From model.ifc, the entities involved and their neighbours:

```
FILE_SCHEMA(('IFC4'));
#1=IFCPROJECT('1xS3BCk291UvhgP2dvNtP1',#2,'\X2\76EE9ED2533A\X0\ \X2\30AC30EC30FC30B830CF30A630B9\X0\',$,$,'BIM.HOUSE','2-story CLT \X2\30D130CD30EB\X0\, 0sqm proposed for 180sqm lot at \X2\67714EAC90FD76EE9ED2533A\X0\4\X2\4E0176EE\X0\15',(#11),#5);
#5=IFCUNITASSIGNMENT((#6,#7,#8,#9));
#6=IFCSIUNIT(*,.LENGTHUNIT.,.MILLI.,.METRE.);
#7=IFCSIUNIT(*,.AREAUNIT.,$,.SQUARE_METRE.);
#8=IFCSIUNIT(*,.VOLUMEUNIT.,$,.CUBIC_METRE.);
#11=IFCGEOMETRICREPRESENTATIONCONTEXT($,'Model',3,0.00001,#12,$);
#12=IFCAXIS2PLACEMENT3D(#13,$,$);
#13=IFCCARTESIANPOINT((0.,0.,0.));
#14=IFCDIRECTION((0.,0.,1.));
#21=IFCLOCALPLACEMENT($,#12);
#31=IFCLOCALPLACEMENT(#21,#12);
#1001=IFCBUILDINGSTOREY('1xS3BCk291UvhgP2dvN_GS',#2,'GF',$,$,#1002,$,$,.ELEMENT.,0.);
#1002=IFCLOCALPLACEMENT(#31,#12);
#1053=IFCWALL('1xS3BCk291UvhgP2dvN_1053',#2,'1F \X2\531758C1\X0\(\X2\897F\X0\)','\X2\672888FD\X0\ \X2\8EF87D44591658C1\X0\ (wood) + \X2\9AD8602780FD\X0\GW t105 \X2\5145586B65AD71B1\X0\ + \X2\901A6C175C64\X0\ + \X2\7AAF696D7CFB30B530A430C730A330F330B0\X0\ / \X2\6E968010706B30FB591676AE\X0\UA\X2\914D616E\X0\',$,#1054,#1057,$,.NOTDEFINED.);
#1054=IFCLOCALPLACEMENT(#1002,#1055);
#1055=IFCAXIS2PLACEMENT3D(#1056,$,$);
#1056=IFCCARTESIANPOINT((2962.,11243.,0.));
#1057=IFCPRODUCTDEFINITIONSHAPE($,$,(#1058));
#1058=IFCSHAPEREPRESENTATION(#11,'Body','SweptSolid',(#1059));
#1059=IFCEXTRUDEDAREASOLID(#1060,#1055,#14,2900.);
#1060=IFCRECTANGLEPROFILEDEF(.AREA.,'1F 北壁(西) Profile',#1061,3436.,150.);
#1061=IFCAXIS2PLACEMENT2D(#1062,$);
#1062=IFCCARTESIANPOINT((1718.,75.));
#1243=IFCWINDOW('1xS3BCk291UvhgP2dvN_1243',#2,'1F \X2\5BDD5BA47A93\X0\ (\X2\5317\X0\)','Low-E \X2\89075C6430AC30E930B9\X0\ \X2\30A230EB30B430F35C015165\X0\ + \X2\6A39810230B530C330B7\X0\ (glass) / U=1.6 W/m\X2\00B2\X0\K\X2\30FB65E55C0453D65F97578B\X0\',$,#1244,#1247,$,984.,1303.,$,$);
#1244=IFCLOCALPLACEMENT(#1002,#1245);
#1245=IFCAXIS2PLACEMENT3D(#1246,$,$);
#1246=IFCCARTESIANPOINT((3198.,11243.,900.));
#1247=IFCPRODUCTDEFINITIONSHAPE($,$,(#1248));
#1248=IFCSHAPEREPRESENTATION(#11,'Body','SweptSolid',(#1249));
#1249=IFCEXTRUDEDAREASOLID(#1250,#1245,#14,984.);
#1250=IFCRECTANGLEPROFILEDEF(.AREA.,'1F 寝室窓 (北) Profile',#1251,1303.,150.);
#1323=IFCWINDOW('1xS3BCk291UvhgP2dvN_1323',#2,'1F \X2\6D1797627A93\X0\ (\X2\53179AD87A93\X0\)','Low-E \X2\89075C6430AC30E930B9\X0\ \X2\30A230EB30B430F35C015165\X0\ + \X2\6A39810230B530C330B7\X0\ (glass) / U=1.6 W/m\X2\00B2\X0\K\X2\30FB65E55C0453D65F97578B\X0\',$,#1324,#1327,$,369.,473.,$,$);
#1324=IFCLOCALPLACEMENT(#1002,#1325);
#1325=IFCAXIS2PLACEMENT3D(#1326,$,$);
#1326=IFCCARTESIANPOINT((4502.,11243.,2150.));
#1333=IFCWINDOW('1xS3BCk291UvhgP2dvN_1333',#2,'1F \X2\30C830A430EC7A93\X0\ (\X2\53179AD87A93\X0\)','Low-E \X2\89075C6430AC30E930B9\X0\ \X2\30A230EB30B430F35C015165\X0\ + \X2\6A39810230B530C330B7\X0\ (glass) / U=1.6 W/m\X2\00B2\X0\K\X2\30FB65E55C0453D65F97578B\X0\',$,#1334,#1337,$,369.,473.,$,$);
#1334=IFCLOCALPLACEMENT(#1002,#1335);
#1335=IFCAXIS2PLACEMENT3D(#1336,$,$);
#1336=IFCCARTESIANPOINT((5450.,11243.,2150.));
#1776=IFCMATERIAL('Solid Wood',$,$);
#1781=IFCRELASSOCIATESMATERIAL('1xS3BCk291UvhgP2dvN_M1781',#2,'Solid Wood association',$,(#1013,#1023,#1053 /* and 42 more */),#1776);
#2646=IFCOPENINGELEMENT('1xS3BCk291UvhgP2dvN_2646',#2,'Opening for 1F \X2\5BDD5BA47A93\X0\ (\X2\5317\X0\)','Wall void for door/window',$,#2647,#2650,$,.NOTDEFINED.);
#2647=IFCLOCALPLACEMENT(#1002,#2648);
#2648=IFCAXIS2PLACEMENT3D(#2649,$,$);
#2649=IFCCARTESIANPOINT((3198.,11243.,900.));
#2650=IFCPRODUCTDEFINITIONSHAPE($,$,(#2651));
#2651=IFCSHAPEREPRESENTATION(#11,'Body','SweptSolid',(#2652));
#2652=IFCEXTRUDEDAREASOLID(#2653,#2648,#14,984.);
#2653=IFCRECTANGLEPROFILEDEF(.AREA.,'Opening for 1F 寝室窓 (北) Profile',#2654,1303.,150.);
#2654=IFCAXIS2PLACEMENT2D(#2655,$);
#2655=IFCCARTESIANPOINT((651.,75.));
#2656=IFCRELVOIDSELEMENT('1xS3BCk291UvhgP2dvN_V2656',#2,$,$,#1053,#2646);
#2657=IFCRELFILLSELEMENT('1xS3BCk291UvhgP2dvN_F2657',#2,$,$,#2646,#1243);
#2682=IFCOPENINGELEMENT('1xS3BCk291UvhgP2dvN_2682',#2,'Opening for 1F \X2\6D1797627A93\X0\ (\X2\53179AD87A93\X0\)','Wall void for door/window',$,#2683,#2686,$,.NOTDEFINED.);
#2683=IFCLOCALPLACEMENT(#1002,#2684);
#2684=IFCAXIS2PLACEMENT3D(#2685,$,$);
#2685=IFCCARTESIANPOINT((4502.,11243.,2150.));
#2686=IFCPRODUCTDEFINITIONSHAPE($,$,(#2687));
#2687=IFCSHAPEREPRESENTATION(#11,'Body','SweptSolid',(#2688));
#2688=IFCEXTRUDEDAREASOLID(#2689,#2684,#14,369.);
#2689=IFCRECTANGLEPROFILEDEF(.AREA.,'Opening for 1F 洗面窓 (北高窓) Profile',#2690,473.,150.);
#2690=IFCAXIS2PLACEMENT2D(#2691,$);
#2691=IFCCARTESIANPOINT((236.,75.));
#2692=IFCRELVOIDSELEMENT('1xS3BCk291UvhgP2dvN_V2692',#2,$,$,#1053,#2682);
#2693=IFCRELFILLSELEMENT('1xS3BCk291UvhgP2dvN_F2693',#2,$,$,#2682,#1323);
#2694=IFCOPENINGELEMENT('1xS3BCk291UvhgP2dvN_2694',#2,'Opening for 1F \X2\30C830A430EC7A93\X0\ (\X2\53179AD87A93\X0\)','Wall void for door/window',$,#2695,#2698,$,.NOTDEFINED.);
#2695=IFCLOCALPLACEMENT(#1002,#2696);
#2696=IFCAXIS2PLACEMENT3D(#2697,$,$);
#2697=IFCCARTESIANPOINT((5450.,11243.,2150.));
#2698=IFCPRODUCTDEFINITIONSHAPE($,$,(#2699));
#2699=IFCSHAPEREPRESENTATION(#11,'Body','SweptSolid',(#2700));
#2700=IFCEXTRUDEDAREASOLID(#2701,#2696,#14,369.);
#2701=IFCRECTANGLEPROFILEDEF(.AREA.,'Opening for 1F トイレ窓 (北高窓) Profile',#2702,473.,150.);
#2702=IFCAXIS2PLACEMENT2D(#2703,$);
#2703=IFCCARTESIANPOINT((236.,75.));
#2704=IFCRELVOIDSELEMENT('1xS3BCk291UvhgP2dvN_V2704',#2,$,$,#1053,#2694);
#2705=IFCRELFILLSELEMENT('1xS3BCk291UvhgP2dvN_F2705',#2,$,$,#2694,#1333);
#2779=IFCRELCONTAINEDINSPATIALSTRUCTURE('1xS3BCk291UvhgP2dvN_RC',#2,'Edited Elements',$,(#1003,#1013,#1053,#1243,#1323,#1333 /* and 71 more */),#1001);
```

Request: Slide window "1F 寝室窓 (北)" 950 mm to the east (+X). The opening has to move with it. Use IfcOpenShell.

```python
import ifcopenshell
import ifcopenshell.api.geometry
import ifcopenshell.util.placement
import ifcopenshell.util.unit

model = ifcopenshell.open("model.ifc")
unit_scale = ifcopenshell.util.unit.calculate_unit_scale(model)

window = model.by_id(1243)
opening = window.FillsVoids[0].RelatingOpeningElement
wall = opening.VoidsElements[0].RelatingBuildingElement

wall_matrix = ifcopenshell.util.placement.get_local_placement(wall.ObjectPlacement)
shift = wall_matrix[:3, 0] * 0.95 / unit_scale
before = ifcopenshell.util.placement.get_local_placement(window.ObjectPlacement)[:3, 3].copy()

# The window is not placed relative to its opening, so move both.
for product in (opening, window):
    matrix = ifcopenshell.util.placement.get_local_placement(product.ObjectPlacement)
    matrix[:3, 3] += shift
    ifcopenshell.api.geometry.edit_object_placement(model, product=product, matrix=matrix, is_si=False)

after = ifcopenshell.util.placement.get_local_placement(window.ObjectPlacement)[:3, 3]
print("window moved by", (after - before).round(3) + 0.0)

model.write("model_edited.ifc")
```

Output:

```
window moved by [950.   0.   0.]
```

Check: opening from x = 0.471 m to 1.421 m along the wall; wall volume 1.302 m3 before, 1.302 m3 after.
